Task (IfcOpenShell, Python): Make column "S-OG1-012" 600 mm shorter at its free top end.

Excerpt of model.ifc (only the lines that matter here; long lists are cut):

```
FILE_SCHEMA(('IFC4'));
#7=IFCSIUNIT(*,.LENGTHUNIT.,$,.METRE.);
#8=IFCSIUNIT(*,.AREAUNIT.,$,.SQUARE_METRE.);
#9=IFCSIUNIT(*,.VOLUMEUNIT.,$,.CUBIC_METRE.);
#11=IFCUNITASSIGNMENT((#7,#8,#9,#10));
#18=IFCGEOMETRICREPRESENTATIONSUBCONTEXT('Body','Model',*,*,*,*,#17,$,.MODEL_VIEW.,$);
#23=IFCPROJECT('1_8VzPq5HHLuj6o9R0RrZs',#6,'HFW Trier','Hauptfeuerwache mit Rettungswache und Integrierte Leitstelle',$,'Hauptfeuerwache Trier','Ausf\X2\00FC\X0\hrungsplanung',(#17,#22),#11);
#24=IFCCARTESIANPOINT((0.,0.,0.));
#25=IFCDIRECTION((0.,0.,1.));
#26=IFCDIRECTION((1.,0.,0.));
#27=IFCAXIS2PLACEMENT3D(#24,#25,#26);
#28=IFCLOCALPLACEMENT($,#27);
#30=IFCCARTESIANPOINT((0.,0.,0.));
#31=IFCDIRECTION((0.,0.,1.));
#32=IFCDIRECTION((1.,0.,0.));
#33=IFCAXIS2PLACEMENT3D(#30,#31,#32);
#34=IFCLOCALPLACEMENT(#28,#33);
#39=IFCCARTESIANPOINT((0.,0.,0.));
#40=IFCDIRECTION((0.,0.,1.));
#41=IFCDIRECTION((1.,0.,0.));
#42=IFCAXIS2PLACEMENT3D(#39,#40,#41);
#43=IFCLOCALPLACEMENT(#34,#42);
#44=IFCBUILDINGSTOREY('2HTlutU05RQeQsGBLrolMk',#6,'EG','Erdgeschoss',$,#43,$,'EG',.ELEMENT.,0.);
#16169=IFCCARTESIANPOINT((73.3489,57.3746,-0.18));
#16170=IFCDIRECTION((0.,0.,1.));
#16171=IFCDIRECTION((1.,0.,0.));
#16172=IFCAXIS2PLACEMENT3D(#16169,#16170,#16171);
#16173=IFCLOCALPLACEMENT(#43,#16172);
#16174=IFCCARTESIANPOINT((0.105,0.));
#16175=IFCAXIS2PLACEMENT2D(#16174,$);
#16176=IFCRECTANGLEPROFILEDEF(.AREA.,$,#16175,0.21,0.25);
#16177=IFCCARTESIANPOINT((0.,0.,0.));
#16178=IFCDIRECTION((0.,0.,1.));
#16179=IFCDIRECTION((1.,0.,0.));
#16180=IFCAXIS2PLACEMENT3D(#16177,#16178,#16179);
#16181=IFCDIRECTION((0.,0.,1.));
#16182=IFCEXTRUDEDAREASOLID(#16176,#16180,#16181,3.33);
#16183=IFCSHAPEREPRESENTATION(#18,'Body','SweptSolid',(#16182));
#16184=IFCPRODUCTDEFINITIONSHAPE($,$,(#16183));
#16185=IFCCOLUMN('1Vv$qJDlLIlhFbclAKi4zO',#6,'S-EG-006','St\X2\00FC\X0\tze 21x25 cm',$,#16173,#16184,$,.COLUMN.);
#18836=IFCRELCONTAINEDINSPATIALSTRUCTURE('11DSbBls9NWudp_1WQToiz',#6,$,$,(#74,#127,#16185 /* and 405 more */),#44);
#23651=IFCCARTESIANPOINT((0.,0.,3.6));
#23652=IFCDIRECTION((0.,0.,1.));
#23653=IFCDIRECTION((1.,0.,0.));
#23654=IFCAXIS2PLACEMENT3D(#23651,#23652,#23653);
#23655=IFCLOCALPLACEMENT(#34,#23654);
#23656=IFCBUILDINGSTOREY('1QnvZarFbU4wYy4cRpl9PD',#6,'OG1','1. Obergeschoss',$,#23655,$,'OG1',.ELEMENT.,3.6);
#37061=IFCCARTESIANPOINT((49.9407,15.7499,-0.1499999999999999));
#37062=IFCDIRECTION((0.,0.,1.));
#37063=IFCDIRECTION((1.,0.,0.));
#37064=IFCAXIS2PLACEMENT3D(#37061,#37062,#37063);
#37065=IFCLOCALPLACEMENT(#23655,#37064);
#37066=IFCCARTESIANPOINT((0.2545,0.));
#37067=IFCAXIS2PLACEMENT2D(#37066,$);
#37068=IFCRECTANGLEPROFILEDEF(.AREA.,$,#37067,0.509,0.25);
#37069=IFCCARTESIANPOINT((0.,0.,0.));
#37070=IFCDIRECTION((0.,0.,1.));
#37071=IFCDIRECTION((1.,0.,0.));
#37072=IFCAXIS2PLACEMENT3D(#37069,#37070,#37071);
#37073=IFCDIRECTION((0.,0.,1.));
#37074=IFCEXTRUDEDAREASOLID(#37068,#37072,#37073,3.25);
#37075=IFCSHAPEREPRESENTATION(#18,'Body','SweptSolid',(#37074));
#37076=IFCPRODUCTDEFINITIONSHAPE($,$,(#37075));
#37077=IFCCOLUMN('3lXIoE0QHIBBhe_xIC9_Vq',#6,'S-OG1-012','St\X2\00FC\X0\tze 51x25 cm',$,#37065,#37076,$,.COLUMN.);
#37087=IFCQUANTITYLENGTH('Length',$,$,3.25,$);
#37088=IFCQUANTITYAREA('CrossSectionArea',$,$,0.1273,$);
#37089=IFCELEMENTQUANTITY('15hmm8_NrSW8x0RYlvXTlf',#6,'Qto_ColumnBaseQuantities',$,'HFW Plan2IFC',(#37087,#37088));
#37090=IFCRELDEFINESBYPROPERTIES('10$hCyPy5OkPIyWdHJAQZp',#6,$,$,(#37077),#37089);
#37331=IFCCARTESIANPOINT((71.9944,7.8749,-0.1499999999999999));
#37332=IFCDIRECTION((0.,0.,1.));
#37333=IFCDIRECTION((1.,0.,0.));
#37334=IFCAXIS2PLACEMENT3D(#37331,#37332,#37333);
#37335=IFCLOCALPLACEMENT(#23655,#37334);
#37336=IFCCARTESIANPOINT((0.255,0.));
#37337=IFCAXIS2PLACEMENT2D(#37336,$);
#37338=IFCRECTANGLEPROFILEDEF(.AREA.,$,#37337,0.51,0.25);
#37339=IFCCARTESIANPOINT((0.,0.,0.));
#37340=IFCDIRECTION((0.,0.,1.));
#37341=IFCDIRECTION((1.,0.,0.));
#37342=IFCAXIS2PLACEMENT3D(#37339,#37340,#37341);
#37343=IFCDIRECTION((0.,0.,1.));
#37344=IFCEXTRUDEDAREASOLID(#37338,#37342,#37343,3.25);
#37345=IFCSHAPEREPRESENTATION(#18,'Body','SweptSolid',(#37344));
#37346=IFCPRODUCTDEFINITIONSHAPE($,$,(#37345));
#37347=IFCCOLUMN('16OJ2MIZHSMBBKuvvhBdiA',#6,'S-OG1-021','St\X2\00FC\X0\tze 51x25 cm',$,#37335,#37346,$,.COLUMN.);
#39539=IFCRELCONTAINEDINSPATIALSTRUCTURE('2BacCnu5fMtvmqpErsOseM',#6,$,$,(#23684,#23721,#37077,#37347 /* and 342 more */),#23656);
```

```python
import ifcopenshell
import ifcopenshell.api.pset
import ifcopenshell.util.element
import ifcopenshell.util.representation
import ifcopenshell.util.unit

model = ifcopenshell.open("model.ifc")
unit_scale = ifcopenshell.util.unit.calculate_unit_scale(model)

member = model.by_guid("3lXIoE0QHIBBhe_xIC9_Vq")
change = -0.6 / unit_scale

# The extrusion runs towards the end named, so only its depth changes.
body = ifcopenshell.util.representation.get_representation(member, "Model", "Body")
solid = body.Items[0]
old_length = solid.Depth
solid.Depth += change

# Update the stored length and volume.
qto = model.by_id(ifcopenshell.util.element.get_pset(member, "Qto_ColumnBaseQuantities", should_inherit=False)["id"])
ifcopenshell.api.pset.edit_qto(model, qto=qto, properties={"Length": solid.Depth})

print(f"length {old_length:g} -> {solid.Depth:g}")

model.write("model-out.ifc")
```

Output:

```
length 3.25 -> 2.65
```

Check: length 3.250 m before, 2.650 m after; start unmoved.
